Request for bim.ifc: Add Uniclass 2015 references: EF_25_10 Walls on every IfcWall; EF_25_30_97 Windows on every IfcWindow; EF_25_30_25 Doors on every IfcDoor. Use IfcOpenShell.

First a look at what the model holds.

```python
import ifcopenshell

model = ifcopenshell.open("bim.ifc")
print(model.schema)
print("classifications:", [c.Name for c in model.by_type("IfcClassification")])
for ifc_class in ("IfcDoor", "IfcRoof", "IfcStair", "IfcWall", "IfcWindow"):
    print(ifc_class, len(model.by_type(ifc_class)))
```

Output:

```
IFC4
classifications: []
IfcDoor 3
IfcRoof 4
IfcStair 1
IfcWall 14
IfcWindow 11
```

```python
import ifcopenshell
import ifcopenshell.api.classification

model = ifcopenshell.open("bim.ifc")

system = ifcopenshell.api.classification.add_classification(model, classification="Uniclass 2015")

codes = {
    "IfcWall": ("EF_25_10", "Walls"),
    "IfcWindow": ("EF_25_30_97", "Windows"),
    "IfcDoor": ("EF_25_30_25", "Doors"),
}
for ifc_class, (code, name) in codes.items():
    products = model.by_type(ifc_class)
    ifcopenshell.api.classification.add_reference(
        model, products=products, classification=system, identification=code, name=name
    )
    print(code, len(products))

model.write("bim_v2.ifc")
```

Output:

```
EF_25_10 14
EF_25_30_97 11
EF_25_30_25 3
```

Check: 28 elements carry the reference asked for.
